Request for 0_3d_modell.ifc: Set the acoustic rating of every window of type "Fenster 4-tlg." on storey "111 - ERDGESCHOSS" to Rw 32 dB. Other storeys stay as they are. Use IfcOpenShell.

First a look at what the model holds.

```python
import ifcopenshell
import ifcopenshell.util.element

model = ifcopenshell.open("0_3d_modell.ifc")
print(model.schema)
storey = next(s for s in model.by_type("IfcBuildingStorey") if s.Name == "111 - ERDGESCHOSS")
windows = [e for e in ifcopenshell.util.element.get_decomposition(storey) if e.is_a("IfcWindow")]
seen = {}
for e in windows:
    element_type = ifcopenshell.util.element.get_type(e)
    key = (element_type.Name if element_type != e and element_type else None, ifcopenshell.util.element.get_pset(e, "Pset_WindowCommon", "AcousticRating"))
    seen[key] = seen.get(key, 0) + 1
for (name, value), count in sorted(seen.items(), key=str):
    print(count, "x", name, "|", value)
```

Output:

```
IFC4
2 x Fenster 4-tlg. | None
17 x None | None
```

```python
import ifcopenshell
import ifcopenshell.api.pset
import ifcopenshell.util.element

model = ifcopenshell.open("0_3d_modell.ifc")

storey = next(s for s in model.by_type("IfcBuildingStorey") if s.Name == "111 - ERDGESCHOSS")
windows = [e for e in ifcopenshell.util.element.get_decomposition(storey) if e.is_a("IfcWindow")]

count = 0
for e in windows:
    element_type = ifcopenshell.util.element.get_type(e)
    if element_type in (None, e) or element_type.Name != "Fenster 4-tlg.":
        continue
    # add_pset returns the element's existing set when there is one.
    pset = ifcopenshell.api.pset.add_pset(model, product=e, name="Pset_WindowCommon")
    ifcopenshell.api.pset.edit_pset(model, pset=pset, properties={"AcousticRating": "Rw 32 dB"})
    count += 1

print(count, "windows updated")

model.write("0_3d_modell_rev.ifc")
```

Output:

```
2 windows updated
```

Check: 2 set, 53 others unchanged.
